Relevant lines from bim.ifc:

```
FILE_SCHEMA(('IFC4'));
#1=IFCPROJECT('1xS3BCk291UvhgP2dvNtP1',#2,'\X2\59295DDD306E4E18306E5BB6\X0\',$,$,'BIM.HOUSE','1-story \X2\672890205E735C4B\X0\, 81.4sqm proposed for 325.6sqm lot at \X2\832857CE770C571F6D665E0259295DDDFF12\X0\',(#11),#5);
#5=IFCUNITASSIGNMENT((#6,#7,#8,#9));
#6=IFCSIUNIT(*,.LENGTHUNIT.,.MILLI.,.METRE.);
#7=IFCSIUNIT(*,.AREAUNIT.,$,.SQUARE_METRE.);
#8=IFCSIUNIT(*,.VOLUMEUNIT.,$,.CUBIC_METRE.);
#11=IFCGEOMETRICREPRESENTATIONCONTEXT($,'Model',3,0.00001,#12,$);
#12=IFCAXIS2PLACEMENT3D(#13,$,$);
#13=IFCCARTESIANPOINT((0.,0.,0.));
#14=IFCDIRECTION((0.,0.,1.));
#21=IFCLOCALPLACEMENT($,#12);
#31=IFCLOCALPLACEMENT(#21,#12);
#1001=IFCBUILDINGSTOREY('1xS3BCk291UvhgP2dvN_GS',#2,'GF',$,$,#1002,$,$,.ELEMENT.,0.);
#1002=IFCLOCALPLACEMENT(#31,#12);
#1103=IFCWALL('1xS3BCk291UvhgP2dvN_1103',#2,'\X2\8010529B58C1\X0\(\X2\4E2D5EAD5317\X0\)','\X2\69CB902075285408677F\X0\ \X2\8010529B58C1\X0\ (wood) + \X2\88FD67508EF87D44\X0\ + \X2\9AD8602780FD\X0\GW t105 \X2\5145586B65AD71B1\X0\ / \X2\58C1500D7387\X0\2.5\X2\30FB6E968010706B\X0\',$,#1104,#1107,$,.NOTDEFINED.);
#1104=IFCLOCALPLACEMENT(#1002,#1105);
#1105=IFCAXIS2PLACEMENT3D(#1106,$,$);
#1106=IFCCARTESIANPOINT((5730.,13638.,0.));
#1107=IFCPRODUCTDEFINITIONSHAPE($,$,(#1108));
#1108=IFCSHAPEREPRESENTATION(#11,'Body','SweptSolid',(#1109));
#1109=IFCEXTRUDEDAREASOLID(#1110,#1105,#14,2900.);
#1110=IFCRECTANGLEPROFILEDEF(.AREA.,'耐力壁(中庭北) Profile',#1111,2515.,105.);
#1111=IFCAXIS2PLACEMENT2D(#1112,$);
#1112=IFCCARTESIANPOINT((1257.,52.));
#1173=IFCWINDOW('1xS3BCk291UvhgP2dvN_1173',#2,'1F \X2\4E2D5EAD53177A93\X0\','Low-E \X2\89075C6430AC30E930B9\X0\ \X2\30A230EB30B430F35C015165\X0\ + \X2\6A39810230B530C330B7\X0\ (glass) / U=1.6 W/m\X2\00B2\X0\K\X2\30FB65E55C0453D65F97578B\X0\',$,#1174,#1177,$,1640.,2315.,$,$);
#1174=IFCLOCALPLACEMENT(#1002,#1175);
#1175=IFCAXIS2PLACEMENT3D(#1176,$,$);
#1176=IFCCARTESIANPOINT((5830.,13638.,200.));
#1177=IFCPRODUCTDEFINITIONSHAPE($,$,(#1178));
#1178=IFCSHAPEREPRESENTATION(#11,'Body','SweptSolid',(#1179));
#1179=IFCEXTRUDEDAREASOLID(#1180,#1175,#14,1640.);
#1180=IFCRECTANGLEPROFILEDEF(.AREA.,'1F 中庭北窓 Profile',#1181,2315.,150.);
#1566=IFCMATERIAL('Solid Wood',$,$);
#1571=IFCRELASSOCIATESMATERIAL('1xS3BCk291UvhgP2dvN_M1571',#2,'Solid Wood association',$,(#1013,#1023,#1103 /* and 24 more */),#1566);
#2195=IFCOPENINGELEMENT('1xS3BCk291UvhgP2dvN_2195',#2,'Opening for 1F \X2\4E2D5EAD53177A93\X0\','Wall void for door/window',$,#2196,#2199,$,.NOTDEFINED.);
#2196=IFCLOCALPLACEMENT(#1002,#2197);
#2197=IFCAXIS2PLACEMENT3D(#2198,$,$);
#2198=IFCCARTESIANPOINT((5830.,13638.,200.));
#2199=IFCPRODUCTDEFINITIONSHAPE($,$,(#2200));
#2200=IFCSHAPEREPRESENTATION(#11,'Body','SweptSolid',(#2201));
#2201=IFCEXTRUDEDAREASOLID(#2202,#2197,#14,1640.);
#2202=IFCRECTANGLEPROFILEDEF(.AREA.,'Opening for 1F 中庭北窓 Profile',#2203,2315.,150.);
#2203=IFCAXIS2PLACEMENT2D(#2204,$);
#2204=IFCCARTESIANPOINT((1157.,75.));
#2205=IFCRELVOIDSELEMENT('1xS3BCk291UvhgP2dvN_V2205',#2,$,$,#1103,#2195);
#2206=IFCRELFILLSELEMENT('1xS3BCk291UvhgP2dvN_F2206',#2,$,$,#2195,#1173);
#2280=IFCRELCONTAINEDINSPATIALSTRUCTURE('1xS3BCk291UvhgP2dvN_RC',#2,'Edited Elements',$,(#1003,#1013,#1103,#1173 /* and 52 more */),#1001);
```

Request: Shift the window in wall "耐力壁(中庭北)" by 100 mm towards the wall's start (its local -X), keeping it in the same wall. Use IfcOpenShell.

```python
import ifcopenshell
import ifcopenshell.api.geometry
import ifcopenshell.util.placement
import ifcopenshell.util.unit

model = ifcopenshell.open("bim.ifc")
unit_scale = ifcopenshell.util.unit.calculate_unit_scale(model)

window = model.by_guid("1xS3BCk291UvhgP2dvN_1173")
opening = window.FillsVoids[0].RelatingOpeningElement
wall = opening.VoidsElements[0].RelatingBuildingElement

wall_matrix = ifcopenshell.util.placement.get_local_placement(wall.ObjectPlacement)
shift = wall_matrix[:3, 0] * -0.1 / unit_scale
before = ifcopenshell.util.placement.get_local_placement(window.ObjectPlacement)[:3, 3].copy()

# The window is not placed relative to its opening, so move both.
for product in (opening, window):
    matrix = ifcopenshell.util.placement.get_local_placement(product.ObjectPlacement)
    matrix[:3, 3] += shift
    ifcopenshell.api.geometry.edit_object_placement(model, product=product, matrix=matrix, is_si=False)

after = ifcopenshell.util.placement.get_local_placement(window.ObjectPlacement)[:3, 3]
print("window moved by", (after - before).round(3) + 0.0)

model.write("bim_v2.ifc")
```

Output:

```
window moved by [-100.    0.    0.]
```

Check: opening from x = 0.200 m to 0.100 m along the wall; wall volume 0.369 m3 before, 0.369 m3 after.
